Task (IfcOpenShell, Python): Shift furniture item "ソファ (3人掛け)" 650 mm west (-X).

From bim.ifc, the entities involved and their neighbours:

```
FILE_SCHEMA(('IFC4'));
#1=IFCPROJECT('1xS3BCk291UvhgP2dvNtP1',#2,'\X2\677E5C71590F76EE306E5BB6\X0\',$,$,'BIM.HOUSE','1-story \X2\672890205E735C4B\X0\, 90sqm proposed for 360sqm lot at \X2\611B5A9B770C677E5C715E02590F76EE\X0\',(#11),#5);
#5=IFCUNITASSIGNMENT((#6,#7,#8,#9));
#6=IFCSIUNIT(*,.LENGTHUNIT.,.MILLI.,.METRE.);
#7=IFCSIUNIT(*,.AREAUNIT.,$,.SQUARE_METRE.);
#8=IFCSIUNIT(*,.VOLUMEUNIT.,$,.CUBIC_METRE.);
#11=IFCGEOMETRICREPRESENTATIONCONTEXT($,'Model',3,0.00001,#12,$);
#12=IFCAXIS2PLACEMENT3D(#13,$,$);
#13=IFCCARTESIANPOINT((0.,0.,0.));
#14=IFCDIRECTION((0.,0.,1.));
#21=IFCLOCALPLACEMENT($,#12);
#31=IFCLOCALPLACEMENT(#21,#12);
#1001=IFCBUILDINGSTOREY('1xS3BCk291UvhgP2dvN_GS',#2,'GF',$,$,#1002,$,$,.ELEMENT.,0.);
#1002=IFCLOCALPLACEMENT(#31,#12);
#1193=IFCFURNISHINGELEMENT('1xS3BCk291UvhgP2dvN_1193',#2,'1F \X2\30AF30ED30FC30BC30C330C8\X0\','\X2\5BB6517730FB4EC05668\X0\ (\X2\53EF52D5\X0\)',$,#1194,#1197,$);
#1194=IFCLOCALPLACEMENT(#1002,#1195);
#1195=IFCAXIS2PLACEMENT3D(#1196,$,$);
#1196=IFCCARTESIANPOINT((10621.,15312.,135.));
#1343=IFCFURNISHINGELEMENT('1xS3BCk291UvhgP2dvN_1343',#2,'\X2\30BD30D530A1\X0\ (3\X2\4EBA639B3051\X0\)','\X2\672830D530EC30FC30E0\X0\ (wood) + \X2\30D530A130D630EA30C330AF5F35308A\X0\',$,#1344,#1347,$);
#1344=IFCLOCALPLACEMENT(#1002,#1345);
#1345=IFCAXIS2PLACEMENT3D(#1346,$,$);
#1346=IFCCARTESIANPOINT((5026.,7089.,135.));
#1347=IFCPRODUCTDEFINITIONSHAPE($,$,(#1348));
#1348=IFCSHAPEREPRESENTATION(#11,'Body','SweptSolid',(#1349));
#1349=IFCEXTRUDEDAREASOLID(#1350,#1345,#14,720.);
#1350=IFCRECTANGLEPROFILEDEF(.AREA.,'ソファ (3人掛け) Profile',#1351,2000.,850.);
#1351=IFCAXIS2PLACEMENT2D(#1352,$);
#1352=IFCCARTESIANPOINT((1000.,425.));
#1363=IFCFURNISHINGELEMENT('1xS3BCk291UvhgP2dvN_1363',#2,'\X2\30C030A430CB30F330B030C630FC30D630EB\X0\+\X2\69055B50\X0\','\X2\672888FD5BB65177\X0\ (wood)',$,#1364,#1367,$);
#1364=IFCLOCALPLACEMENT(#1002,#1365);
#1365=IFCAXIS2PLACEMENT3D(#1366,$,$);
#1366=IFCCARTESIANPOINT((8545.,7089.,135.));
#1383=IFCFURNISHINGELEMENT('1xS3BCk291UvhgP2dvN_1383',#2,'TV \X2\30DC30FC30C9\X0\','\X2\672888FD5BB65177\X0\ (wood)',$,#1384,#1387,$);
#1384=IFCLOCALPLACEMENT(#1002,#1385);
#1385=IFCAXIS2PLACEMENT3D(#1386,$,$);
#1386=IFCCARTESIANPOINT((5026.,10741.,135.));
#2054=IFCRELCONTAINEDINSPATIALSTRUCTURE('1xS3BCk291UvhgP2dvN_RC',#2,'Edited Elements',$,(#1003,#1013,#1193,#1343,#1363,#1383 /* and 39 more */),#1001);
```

```python
import ifcopenshell
import ifcopenshell.api.geometry
import ifcopenshell.util.placement
import ifcopenshell.util.unit

model = ifcopenshell.open("bim.ifc")
unit_scale = ifcopenshell.util.unit.calculate_unit_scale(model)

item = model.by_guid("1xS3BCk291UvhgP2dvN_1343")
matrix = ifcopenshell.util.placement.get_local_placement(item.ObjectPlacement)
matrix[0, 3] -= 0.65 / unit_scale
ifcopenshell.api.geometry.edit_object_placement(model, product=item, matrix=matrix, is_si=False)

print(ifcopenshell.util.placement.get_local_placement(item.ObjectPlacement).round(3) + 0.0)

model.write("bim_updated.ifc")
```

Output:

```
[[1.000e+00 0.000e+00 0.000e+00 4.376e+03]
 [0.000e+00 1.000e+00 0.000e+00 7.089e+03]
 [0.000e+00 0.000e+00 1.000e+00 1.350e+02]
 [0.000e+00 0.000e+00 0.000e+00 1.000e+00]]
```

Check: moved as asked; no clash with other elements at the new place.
